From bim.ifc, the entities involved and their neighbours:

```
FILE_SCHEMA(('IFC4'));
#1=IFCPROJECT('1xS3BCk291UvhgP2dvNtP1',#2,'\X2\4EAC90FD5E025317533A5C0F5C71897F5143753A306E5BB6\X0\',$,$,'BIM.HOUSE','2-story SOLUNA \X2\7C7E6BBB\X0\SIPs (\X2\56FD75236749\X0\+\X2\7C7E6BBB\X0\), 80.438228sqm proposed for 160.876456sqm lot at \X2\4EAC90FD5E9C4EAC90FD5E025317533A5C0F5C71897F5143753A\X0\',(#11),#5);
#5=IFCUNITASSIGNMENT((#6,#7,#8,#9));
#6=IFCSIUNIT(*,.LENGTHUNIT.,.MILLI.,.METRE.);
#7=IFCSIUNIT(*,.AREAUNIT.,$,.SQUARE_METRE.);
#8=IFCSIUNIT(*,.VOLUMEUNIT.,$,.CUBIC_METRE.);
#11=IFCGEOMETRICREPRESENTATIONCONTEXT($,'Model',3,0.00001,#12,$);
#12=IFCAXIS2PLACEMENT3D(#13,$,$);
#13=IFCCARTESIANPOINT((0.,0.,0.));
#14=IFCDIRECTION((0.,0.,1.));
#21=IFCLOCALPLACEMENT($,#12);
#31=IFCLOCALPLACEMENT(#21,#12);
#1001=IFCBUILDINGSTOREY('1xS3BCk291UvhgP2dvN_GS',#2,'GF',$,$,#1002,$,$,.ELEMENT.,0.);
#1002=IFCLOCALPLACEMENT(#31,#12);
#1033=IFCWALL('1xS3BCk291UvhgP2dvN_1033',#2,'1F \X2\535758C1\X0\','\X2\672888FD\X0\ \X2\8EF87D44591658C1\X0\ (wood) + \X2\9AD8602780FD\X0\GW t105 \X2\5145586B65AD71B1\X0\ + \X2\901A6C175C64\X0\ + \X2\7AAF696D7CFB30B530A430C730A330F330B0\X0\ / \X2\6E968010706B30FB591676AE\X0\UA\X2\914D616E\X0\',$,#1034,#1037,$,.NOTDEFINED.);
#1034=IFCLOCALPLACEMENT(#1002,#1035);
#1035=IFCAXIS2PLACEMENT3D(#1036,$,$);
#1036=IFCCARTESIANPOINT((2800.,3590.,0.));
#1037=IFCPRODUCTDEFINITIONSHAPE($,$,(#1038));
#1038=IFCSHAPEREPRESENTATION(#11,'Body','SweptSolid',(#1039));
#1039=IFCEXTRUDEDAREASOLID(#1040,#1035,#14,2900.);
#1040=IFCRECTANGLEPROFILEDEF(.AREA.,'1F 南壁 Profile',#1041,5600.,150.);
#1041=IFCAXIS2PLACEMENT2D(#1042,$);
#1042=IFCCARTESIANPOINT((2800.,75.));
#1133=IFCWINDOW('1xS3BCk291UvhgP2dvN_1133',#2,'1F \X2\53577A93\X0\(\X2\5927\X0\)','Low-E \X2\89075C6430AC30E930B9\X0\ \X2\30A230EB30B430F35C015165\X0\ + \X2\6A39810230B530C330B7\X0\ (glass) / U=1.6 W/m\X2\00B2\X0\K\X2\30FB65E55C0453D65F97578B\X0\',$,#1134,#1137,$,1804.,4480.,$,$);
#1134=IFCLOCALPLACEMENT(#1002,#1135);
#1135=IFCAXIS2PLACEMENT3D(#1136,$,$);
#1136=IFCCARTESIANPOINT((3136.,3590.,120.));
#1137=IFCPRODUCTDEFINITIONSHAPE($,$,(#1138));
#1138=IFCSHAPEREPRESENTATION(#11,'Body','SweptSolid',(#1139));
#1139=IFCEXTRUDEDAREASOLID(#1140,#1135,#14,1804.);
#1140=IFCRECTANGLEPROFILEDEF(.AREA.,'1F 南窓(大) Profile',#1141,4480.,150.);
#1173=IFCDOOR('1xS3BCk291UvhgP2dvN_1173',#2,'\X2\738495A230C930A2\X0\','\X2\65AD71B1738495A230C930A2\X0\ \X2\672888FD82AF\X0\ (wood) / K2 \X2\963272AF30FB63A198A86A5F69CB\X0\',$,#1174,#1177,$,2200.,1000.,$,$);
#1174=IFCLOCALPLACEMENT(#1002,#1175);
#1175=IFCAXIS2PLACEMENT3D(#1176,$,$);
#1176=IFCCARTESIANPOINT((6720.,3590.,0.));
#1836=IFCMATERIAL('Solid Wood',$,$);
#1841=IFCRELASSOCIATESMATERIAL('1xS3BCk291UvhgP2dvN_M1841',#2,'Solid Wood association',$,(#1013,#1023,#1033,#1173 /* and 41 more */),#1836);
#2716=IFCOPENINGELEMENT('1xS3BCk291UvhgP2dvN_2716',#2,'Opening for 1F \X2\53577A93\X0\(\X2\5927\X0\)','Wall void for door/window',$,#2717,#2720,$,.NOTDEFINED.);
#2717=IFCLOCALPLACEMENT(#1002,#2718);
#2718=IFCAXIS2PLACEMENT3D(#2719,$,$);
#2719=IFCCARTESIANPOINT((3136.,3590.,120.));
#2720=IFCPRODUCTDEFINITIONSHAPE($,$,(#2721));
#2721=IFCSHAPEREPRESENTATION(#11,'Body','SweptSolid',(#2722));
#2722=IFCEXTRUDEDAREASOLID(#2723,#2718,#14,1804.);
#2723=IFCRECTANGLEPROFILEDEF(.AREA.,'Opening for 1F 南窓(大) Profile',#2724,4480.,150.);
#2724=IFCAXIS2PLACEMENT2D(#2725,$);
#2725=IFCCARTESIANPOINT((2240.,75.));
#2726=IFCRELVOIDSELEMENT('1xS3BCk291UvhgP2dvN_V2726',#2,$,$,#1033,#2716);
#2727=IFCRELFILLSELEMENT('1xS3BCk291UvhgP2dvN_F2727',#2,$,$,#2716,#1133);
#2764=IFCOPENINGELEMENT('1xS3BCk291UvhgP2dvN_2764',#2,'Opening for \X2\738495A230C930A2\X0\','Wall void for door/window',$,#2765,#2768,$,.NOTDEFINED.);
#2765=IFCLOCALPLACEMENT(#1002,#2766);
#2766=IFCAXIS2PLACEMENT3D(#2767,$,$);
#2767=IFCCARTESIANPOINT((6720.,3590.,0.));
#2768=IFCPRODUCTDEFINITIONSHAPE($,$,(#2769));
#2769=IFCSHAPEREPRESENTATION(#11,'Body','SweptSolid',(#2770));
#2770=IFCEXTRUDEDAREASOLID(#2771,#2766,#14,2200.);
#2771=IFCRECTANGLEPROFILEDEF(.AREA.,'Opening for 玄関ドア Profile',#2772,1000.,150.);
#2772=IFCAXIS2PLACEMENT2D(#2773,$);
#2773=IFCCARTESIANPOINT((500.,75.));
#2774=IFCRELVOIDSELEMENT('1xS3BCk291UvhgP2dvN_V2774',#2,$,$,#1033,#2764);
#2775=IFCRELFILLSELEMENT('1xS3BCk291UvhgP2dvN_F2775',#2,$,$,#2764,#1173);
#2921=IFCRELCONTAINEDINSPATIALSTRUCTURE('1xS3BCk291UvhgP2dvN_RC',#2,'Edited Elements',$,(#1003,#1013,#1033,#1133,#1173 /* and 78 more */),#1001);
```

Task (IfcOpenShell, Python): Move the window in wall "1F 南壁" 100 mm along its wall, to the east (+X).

```python
import ifcopenshell
import ifcopenshell.api.geometry
import ifcopenshell.util.placement
import ifcopenshell.util.unit

model = ifcopenshell.open("bim.ifc")
unit_scale = ifcopenshell.util.unit.calculate_unit_scale(model)

window = model.by_guid("1xS3BCk291UvhgP2dvN_1133")
opening = window.FillsVoids[0].RelatingOpeningElement
wall = opening.VoidsElements[0].RelatingBuildingElement

wall_matrix = ifcopenshell.util.placement.get_local_placement(wall.ObjectPlacement)
shift = wall_matrix[:3, 0] * 0.1 / unit_scale
before = ifcopenshell.util.placement.get_local_placement(window.ObjectPlacement)[:3, 3].copy()

# The window is not placed relative to its opening, so move both.
for product in (opening, window):
    matrix = ifcopenshell.util.placement.get_local_placement(product.ObjectPlacement)
    matrix[:3, 3] += shift
    ifcopenshell.api.geometry.edit_object_placement(model, product=product, matrix=matrix, is_si=False)

after = ifcopenshell.util.placement.get_local_placement(window.ObjectPlacement)[:3, 3]
print("window moved by", (after - before).round(3) + 0.0)

model.write("bim_updated.ifc")
```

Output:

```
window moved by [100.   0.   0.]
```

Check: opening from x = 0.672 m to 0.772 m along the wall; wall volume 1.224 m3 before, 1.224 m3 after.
